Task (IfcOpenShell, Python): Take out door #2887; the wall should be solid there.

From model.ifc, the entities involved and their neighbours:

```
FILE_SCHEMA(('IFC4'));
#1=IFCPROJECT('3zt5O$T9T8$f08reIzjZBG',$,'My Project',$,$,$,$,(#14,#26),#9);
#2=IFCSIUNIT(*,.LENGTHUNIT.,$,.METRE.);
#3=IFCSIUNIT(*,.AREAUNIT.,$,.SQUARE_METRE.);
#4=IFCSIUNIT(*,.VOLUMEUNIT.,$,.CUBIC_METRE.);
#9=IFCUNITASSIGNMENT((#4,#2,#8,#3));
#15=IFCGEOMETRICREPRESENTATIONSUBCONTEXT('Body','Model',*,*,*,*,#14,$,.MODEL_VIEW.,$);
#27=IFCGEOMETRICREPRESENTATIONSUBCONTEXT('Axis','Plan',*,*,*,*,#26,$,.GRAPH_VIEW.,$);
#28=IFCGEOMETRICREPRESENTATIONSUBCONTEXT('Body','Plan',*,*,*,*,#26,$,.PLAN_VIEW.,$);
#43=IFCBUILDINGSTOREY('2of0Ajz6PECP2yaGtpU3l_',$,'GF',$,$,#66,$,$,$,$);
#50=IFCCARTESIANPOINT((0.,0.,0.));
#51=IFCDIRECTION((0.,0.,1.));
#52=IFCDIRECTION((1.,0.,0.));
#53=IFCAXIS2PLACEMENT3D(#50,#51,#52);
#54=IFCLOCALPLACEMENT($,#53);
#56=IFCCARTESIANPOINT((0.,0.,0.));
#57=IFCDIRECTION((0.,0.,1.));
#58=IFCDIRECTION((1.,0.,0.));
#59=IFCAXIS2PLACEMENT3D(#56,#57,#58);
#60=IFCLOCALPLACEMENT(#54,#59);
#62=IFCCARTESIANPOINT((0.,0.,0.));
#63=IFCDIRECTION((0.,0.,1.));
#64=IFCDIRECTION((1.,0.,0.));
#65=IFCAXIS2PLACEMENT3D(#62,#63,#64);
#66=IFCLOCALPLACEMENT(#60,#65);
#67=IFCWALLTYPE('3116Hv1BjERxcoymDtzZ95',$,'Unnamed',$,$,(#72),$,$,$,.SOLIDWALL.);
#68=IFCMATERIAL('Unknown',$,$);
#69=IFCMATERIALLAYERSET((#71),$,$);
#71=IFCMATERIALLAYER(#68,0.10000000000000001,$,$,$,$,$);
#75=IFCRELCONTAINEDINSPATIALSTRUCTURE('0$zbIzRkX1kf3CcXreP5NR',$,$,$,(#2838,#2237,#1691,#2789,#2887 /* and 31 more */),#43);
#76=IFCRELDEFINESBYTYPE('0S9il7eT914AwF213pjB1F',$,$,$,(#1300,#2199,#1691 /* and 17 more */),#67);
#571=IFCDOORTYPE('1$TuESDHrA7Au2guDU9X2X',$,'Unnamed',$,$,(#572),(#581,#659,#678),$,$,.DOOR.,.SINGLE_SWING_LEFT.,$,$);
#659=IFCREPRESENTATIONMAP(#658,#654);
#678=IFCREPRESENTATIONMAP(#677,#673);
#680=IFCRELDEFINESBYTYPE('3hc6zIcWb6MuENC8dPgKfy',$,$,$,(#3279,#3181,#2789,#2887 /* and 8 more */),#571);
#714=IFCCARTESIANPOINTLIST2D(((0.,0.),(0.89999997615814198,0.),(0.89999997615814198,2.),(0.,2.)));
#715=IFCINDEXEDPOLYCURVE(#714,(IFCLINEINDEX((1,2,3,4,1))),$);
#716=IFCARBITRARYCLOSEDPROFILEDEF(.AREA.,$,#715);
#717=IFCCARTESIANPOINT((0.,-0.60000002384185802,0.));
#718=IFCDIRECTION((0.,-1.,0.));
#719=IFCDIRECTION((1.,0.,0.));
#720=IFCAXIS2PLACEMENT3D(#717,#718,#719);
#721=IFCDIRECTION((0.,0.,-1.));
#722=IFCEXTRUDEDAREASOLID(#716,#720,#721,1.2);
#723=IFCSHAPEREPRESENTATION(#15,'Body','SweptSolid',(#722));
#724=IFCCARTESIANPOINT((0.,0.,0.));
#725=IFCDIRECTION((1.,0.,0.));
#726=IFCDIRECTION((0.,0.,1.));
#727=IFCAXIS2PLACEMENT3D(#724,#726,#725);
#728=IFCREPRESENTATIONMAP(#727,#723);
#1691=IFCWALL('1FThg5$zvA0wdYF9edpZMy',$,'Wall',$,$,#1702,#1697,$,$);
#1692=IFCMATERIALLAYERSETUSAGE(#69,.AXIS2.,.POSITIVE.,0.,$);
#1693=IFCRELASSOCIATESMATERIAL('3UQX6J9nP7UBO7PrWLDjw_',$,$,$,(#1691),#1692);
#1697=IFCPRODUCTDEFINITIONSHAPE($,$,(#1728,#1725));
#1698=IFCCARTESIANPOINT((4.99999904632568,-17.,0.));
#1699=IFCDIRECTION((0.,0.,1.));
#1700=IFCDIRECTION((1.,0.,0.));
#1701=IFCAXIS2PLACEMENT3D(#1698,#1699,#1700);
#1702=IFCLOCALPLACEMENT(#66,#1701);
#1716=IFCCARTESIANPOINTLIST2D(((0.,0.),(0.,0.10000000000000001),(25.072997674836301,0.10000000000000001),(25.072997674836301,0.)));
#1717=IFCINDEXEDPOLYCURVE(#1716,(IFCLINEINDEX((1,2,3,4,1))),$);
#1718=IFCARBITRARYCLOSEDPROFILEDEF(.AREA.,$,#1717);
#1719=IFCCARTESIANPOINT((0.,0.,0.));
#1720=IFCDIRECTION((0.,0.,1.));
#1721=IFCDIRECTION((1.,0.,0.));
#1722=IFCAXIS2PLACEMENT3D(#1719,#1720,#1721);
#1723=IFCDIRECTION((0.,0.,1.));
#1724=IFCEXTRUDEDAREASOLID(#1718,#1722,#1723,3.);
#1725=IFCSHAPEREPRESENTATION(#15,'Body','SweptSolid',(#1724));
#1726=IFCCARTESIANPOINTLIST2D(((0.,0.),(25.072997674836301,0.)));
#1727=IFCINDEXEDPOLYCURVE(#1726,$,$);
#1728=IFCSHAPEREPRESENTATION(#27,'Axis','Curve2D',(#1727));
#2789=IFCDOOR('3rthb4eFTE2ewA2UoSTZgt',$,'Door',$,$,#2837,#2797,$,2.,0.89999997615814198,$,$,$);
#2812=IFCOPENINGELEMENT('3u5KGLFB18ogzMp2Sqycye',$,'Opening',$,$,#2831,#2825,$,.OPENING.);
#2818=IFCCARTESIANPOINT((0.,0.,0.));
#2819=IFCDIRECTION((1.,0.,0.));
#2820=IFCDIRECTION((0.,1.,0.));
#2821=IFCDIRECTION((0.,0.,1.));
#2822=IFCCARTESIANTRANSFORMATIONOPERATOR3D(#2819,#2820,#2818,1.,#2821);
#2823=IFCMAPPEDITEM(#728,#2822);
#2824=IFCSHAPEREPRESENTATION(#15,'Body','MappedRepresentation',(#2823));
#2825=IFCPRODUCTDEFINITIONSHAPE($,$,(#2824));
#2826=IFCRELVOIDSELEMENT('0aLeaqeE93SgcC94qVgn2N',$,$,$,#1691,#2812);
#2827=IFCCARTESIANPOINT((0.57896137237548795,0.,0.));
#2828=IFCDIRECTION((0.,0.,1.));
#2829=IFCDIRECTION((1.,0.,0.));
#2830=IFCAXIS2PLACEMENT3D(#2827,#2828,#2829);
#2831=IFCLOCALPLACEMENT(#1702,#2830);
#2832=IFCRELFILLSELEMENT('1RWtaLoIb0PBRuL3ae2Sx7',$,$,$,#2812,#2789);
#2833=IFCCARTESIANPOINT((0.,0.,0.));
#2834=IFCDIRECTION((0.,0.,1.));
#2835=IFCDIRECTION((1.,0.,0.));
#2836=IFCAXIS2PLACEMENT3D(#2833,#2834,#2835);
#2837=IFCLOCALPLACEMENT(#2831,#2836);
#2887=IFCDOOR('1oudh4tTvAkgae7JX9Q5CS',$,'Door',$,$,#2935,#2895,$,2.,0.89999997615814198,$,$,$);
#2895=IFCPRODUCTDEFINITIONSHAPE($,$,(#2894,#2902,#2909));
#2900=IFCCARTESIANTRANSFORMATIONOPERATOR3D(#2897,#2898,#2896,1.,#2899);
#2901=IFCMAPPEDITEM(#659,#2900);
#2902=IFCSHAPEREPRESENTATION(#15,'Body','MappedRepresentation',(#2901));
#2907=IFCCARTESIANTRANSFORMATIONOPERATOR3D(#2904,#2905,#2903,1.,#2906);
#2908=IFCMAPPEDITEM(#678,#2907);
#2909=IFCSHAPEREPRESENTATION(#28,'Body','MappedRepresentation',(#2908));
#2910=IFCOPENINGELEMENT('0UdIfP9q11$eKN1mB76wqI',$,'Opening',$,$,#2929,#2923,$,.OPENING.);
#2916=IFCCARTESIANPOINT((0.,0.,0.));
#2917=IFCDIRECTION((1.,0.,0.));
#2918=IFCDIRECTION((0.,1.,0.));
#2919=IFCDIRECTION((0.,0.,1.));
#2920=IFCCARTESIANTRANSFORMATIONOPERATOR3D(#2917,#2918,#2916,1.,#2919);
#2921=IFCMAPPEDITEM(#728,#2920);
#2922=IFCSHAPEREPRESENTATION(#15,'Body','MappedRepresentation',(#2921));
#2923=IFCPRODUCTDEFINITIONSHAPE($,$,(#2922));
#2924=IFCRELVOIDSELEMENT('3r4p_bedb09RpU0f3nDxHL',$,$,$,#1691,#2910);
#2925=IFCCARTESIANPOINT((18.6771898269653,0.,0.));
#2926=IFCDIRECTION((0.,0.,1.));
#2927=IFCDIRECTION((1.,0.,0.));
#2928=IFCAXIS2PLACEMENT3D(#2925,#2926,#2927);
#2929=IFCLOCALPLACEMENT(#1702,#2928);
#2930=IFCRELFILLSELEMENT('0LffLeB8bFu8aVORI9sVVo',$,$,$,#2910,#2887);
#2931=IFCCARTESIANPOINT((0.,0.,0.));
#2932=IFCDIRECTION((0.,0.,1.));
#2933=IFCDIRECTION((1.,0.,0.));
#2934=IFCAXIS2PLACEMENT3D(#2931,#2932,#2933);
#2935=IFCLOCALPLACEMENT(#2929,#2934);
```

```python
import ifcopenshell
import ifcopenshell.api.feature
import ifcopenshell.api.root
import ifcopenshell.geom
import ifcopenshell.util.shape

model = ifcopenshell.open("model.ifc")
settings = ifcopenshell.geom.settings()


def volume(element):
    """Net volume in cubic metres, openings subtracted."""
    shape = ifcopenshell.geom.create_shape(settings, element)
    return ifcopenshell.util.shape.get_volume(shape.geometry)


door = model.by_guid("1oudh4tTvAkgae7JX9Q5CS")
opening = door.FillsVoids[0].RelatingOpeningElement
wall = opening.VoidsElements[0].RelatingBuildingElement
before = volume(wall)

ifcopenshell.api.root.remove_product(model, product=door)
ifcopenshell.api.feature.remove_feature(model, feature=opening)

after = volume(wall)

print(f"wall volume {before:.3f} -> {after:.3f} m3")

model.write("model-out.ifc")
```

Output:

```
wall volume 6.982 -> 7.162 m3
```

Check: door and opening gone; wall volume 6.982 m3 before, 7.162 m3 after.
